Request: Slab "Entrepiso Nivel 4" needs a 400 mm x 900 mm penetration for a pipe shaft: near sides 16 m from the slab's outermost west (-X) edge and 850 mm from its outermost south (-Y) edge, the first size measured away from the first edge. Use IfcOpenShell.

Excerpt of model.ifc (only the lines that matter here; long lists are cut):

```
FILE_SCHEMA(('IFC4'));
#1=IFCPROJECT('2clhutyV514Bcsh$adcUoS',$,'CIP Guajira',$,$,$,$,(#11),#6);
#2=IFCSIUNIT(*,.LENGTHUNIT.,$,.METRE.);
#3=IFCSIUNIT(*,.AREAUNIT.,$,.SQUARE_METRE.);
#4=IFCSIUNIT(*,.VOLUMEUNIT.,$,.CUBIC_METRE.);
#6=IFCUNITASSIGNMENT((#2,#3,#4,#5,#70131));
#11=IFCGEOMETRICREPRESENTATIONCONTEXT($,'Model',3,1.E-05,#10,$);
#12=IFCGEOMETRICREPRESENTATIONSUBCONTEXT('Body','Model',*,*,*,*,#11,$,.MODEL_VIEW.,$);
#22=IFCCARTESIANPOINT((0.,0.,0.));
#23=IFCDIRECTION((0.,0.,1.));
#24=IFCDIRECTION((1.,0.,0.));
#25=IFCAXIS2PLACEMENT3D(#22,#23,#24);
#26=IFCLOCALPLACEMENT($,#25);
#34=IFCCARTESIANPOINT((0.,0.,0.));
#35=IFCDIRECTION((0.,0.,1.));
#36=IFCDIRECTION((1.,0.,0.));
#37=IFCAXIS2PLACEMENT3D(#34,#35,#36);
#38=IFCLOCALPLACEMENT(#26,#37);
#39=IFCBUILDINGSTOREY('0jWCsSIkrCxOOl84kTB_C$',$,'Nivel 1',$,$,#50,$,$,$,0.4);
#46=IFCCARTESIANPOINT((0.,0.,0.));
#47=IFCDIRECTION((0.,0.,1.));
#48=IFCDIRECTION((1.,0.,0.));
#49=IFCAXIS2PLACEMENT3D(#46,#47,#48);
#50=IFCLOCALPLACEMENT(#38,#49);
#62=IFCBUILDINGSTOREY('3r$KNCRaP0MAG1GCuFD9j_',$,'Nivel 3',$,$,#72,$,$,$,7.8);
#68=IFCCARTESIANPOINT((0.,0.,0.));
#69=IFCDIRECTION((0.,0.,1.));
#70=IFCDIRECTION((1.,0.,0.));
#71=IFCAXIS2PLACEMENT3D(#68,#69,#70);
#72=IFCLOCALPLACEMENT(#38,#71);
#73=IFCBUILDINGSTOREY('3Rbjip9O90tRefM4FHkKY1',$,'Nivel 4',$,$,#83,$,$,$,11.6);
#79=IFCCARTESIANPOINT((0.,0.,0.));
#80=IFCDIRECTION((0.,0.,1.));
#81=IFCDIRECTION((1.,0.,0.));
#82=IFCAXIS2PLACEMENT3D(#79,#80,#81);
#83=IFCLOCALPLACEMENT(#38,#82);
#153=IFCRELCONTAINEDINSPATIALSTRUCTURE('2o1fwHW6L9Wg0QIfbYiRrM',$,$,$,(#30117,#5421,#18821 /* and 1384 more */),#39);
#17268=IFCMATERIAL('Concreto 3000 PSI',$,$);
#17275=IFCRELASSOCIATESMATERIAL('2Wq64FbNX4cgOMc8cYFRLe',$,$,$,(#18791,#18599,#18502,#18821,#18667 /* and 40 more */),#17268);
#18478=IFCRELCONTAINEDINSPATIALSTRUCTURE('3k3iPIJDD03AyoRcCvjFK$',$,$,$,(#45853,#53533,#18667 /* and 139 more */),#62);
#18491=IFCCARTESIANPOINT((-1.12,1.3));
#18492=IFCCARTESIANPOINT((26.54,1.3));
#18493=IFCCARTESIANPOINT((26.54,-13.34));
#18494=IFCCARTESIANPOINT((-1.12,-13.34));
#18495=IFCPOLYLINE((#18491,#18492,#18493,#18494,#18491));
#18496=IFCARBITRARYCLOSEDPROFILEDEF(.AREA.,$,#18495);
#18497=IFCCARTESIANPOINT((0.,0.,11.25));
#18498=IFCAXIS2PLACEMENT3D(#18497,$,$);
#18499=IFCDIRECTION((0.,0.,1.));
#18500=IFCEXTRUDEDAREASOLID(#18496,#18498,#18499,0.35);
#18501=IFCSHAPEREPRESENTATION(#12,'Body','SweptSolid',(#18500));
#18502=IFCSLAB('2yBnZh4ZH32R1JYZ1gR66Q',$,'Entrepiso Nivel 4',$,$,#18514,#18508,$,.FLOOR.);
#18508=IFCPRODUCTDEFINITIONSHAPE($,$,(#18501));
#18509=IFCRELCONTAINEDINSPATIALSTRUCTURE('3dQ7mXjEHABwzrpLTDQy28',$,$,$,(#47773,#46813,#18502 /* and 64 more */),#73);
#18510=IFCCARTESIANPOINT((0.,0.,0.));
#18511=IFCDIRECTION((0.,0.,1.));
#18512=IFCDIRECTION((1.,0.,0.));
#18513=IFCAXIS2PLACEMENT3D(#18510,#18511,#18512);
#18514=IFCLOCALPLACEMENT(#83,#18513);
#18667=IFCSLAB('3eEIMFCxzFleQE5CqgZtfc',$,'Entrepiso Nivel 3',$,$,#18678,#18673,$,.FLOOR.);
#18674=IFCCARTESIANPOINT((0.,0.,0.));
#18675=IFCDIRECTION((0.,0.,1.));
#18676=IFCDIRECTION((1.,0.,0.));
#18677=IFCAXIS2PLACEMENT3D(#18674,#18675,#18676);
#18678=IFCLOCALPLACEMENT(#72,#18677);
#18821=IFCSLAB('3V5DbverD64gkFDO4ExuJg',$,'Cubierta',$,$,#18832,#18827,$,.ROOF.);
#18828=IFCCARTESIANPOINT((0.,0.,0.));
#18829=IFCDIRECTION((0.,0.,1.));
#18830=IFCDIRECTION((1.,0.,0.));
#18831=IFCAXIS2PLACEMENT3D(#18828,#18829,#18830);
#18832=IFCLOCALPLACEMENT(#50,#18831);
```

```python
import numpy as np
import ifcopenshell
import ifcopenshell.api.feature
import ifcopenshell.api.geometry
import ifcopenshell.api.root
import ifcopenshell.geom
import ifcopenshell.util.placement
import ifcopenshell.util.representation
import ifcopenshell.util.shape
import ifcopenshell.util.unit

model = ifcopenshell.open("model.ifc")
unit_scale = ifcopenshell.util.unit.calculate_unit_scale(model)
settings = ifcopenshell.geom.settings()


def volume(element):
    """Net volume in cubic metres, openings subtracted."""
    shape = ifcopenshell.geom.create_shape(settings, element)
    return ifcopenshell.util.shape.get_volume(shape.geometry)


slab = model.by_guid("2yBnZh4ZH32R1JYZ1gR66Q")
before = volume(slab)

# Extent in the slab's own axes, in metres. The edges named are its -X and -Y sides.
slab_shape = ifcopenshell.geom.create_shape(settings, slab)
vertices = ifcopenshell.util.shape.get_vertices(slab_shape.geometry)
x_min, y_min, bottom = vertices.min(axis=0)
top = vertices[:, 2].max()

opening = ifcopenshell.api.root.create_entity(model, ifc_class="IfcOpeningElement", name="Pipe shaft opening", predefined_type="OPENING")
context = ifcopenshell.util.representation.get_context(model, "Model", "Body", "MODEL_VIEW")
width, depth = 0.4, 0.9
outline = [(0.0, 0.0), (width, 0.0), (width, depth), (0.0, depth), (0.0, 0.0)]
# Overshoot both faces by 50 mm so the cut is clean.
shape = ifcopenshell.api.geometry.add_slab_representation(
    model, context=context, depth=top - bottom + 0.1, polyline=outline
)
ifcopenshell.api.geometry.assign_representation(model, product=opening, representation=shape)

matrix = ifcopenshell.util.placement.get_local_placement(slab.ObjectPlacement)
matrix[:, 3] = matrix @ np.append(np.array([x_min + 16, y_min + 0.85, bottom - 0.05]) / unit_scale, 1.0)
ifcopenshell.api.geometry.edit_object_placement(model, product=opening, matrix=matrix, is_si=False)
ifcopenshell.api.feature.add_feature(model, feature=opening, element=slab)

after = volume(slab)

print(f"slab volume {before:.3f} -> {after:.3f} m3")

model.write("model-out.ifc")
```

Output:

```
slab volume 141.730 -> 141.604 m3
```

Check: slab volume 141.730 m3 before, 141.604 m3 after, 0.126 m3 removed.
